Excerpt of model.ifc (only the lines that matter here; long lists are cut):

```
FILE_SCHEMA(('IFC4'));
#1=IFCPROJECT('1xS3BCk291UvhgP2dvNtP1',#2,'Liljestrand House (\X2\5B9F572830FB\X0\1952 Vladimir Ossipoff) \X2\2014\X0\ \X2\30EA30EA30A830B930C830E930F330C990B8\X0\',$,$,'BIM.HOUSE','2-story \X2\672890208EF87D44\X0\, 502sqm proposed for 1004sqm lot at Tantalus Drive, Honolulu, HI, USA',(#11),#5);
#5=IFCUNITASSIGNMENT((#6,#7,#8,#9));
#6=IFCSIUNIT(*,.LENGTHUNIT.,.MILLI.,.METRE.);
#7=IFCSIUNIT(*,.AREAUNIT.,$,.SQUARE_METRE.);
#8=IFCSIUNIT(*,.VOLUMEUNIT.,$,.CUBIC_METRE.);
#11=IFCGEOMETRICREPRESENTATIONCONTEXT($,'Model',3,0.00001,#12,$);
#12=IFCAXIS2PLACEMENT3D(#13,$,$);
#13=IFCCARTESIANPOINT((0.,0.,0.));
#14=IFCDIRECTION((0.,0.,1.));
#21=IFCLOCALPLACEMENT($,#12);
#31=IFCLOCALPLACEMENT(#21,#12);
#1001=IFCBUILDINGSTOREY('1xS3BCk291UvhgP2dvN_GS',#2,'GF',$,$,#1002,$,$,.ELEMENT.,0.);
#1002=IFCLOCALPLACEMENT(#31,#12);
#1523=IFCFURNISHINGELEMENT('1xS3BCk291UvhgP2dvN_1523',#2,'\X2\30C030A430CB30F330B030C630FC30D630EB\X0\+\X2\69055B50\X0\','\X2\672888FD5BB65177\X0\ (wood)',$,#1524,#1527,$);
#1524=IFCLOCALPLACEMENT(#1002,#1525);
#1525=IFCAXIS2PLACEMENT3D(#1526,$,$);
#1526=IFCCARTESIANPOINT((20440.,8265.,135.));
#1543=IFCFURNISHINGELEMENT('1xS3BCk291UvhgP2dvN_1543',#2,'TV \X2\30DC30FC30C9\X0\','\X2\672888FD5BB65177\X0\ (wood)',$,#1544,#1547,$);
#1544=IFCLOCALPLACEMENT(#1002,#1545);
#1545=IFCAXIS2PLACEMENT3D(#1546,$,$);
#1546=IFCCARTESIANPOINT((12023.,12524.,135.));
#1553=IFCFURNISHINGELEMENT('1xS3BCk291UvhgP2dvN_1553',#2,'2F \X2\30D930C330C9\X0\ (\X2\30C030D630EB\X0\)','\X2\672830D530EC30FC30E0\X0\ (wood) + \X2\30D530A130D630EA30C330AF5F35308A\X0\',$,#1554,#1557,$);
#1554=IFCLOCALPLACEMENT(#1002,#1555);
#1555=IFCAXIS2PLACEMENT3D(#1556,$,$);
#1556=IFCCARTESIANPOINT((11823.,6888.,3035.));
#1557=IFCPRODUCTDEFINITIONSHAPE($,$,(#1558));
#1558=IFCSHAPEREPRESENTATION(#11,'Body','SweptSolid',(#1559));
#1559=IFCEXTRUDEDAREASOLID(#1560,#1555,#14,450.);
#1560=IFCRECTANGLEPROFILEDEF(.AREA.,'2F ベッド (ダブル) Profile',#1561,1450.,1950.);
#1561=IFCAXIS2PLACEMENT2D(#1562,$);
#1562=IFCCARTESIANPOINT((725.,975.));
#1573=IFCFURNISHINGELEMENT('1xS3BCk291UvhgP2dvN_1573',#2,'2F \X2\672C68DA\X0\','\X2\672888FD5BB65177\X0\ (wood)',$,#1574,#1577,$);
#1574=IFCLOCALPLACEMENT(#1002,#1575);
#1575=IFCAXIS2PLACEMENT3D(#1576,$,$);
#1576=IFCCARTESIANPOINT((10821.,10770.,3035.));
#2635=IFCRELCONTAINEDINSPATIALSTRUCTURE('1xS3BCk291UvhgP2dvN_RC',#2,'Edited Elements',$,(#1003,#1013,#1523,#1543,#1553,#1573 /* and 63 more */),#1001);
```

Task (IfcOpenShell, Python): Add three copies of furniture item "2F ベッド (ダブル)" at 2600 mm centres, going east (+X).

```python
import numpy as np
import ifcopenshell
import ifcopenshell.api.geometry
import ifcopenshell.api.root
import ifcopenshell.util.element
import ifcopenshell.util.placement
import ifcopenshell.util.unit

model = ifcopenshell.open("model.ifc")
unit_scale = ifcopenshell.util.unit.calculate_unit_scale(model)


def reuse_history(source, copy):
    """copy_class also copies each property set's owner history, people and application; keep the originals."""
    for rel in copy.IsDefinedBy:
        if rel.is_a("IfcRelDefinesByProperties") and (history := rel.RelatingPropertyDefinition.OwnerHistory):
            rel.RelatingPropertyDefinition.OwnerHistory = source.OwnerHistory
            ifcopenshell.util.element.remove_deep2(model, history)


source = model.by_guid("1xS3BCk291UvhgP2dvN_1553")
base = ifcopenshell.util.placement.get_local_placement(source.ObjectPlacement)
step = np.array([1.0, 0.0, 0.0]) * 2.6 / unit_scale

for i in range(1, 4):
    copy = ifcopenshell.api.root.copy_class(model, product=source)
    copy.Representation = ifcopenshell.util.element.copy_deep(
        model, source.Representation, exclude=["IfcGeometricRepresentationContext", "IfcRepresentationMap"]
    )
    reuse_history(source, copy)
    matrix = base.copy()
    matrix[:3, 3] += i * step
    print("added at", matrix[:3, 3].round(3) + 0.0)
    ifcopenshell.api.geometry.edit_object_placement(model, product=copy, matrix=matrix, is_si=False)

model.write("model_v2.ifc")
```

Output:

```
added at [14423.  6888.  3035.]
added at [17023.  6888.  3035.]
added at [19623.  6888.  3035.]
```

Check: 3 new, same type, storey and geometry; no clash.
